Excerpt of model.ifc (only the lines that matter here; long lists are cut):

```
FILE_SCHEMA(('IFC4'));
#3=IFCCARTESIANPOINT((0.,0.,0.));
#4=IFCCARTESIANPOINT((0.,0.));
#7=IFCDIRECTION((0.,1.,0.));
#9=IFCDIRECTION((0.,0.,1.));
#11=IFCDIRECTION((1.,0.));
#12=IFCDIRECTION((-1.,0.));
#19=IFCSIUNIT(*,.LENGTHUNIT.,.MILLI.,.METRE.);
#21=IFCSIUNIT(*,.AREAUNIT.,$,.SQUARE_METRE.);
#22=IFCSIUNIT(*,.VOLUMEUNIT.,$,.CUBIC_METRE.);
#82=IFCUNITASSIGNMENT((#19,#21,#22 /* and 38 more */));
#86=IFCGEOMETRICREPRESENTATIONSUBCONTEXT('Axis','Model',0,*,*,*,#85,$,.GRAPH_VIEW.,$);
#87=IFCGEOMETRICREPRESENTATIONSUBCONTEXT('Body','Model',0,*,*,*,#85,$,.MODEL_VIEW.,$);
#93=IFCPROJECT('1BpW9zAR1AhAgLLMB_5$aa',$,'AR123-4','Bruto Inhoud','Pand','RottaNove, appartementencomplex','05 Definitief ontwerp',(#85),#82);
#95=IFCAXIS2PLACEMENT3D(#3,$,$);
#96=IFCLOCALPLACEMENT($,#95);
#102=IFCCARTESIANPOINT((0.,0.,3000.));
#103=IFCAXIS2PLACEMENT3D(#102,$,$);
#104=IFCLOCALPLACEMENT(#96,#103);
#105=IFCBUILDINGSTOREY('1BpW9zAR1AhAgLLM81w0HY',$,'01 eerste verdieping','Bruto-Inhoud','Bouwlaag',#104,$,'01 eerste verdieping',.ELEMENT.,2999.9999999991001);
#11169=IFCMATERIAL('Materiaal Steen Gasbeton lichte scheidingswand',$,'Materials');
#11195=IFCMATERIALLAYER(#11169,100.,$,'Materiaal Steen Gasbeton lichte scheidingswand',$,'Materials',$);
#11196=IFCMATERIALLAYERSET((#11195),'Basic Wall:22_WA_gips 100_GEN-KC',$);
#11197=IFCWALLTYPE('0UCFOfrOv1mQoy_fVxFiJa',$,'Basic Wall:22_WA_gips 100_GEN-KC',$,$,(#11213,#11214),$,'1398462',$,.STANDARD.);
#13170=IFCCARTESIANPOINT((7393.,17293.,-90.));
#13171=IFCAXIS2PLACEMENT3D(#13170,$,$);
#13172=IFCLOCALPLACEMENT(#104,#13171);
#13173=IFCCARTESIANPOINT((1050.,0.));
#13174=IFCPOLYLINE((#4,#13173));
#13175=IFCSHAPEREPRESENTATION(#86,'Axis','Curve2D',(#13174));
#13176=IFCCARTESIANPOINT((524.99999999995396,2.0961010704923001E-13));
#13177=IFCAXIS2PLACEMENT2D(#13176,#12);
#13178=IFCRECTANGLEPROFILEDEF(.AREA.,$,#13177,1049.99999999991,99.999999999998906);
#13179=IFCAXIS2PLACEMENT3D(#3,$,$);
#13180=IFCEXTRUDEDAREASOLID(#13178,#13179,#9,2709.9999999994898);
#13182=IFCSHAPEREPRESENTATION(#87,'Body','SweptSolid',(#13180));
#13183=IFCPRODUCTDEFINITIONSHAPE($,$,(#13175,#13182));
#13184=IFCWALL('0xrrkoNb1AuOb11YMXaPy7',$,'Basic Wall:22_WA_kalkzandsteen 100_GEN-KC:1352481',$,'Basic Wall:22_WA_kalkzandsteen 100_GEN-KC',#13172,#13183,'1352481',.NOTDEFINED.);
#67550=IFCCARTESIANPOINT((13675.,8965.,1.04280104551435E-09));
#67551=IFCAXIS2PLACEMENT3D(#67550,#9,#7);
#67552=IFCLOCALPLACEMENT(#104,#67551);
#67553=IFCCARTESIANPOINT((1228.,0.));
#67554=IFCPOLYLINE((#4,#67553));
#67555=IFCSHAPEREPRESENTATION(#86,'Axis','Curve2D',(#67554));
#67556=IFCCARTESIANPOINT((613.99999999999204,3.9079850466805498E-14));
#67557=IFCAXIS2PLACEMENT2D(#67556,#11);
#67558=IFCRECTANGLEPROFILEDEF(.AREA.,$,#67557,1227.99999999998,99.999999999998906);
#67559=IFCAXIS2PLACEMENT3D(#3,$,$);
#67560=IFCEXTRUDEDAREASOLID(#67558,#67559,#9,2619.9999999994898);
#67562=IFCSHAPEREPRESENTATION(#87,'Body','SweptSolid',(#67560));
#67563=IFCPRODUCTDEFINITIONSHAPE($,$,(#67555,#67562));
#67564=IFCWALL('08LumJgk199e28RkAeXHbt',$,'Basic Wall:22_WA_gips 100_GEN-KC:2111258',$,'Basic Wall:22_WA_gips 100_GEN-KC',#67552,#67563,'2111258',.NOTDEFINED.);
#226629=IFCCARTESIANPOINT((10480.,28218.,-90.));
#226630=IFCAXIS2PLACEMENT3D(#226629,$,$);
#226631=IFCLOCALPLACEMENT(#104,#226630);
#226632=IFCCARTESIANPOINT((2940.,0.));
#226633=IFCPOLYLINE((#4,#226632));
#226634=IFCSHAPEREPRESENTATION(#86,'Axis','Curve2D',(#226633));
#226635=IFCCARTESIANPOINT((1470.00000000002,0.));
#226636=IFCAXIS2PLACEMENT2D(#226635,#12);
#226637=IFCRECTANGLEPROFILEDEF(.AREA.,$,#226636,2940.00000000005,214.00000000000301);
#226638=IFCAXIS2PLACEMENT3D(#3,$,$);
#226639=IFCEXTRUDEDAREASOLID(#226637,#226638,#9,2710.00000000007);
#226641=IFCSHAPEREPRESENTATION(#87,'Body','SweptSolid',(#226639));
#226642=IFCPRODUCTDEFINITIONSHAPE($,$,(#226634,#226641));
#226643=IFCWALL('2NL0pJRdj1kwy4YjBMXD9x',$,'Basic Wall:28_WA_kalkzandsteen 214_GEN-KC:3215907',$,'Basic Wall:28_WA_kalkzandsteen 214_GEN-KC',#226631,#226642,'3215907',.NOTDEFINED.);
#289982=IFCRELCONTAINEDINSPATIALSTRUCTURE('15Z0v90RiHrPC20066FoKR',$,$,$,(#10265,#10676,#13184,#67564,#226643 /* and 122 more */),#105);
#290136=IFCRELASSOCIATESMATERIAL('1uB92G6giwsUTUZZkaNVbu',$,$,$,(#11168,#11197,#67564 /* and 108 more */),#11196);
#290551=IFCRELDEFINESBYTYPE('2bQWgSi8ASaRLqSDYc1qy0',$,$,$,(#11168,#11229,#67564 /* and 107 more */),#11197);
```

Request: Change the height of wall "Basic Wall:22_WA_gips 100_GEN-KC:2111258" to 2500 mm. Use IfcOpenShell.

```python
import ifcopenshell
import ifcopenshell.geom
import ifcopenshell.util.representation
import ifcopenshell.util.shape
import ifcopenshell.util.unit

model = ifcopenshell.open("model.ifc")
unit_scale = ifcopenshell.util.unit.calculate_unit_scale(model)
settings = ifcopenshell.geom.settings()


def volume(element):
    """Net volume in cubic metres, openings subtracted."""
    shape = ifcopenshell.geom.create_shape(settings, element)
    return ifcopenshell.util.shape.get_volume(shape.geometry)


wall = model.by_id(67564)
before = volume(wall)

body = ifcopenshell.util.representation.get_representation(wall, "Model", "Body")
solid = body.Items[0]
old_height = solid.Depth
solid.Depth = 2.5 / unit_scale
after = volume(wall)

print(f"height {old_height:g} -> {solid.Depth:g}, volume {before:.3f} -> {after:.3f} m3")

model.write("model_rev.ifc")
```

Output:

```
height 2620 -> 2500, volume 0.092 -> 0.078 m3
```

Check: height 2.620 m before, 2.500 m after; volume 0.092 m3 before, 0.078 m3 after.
